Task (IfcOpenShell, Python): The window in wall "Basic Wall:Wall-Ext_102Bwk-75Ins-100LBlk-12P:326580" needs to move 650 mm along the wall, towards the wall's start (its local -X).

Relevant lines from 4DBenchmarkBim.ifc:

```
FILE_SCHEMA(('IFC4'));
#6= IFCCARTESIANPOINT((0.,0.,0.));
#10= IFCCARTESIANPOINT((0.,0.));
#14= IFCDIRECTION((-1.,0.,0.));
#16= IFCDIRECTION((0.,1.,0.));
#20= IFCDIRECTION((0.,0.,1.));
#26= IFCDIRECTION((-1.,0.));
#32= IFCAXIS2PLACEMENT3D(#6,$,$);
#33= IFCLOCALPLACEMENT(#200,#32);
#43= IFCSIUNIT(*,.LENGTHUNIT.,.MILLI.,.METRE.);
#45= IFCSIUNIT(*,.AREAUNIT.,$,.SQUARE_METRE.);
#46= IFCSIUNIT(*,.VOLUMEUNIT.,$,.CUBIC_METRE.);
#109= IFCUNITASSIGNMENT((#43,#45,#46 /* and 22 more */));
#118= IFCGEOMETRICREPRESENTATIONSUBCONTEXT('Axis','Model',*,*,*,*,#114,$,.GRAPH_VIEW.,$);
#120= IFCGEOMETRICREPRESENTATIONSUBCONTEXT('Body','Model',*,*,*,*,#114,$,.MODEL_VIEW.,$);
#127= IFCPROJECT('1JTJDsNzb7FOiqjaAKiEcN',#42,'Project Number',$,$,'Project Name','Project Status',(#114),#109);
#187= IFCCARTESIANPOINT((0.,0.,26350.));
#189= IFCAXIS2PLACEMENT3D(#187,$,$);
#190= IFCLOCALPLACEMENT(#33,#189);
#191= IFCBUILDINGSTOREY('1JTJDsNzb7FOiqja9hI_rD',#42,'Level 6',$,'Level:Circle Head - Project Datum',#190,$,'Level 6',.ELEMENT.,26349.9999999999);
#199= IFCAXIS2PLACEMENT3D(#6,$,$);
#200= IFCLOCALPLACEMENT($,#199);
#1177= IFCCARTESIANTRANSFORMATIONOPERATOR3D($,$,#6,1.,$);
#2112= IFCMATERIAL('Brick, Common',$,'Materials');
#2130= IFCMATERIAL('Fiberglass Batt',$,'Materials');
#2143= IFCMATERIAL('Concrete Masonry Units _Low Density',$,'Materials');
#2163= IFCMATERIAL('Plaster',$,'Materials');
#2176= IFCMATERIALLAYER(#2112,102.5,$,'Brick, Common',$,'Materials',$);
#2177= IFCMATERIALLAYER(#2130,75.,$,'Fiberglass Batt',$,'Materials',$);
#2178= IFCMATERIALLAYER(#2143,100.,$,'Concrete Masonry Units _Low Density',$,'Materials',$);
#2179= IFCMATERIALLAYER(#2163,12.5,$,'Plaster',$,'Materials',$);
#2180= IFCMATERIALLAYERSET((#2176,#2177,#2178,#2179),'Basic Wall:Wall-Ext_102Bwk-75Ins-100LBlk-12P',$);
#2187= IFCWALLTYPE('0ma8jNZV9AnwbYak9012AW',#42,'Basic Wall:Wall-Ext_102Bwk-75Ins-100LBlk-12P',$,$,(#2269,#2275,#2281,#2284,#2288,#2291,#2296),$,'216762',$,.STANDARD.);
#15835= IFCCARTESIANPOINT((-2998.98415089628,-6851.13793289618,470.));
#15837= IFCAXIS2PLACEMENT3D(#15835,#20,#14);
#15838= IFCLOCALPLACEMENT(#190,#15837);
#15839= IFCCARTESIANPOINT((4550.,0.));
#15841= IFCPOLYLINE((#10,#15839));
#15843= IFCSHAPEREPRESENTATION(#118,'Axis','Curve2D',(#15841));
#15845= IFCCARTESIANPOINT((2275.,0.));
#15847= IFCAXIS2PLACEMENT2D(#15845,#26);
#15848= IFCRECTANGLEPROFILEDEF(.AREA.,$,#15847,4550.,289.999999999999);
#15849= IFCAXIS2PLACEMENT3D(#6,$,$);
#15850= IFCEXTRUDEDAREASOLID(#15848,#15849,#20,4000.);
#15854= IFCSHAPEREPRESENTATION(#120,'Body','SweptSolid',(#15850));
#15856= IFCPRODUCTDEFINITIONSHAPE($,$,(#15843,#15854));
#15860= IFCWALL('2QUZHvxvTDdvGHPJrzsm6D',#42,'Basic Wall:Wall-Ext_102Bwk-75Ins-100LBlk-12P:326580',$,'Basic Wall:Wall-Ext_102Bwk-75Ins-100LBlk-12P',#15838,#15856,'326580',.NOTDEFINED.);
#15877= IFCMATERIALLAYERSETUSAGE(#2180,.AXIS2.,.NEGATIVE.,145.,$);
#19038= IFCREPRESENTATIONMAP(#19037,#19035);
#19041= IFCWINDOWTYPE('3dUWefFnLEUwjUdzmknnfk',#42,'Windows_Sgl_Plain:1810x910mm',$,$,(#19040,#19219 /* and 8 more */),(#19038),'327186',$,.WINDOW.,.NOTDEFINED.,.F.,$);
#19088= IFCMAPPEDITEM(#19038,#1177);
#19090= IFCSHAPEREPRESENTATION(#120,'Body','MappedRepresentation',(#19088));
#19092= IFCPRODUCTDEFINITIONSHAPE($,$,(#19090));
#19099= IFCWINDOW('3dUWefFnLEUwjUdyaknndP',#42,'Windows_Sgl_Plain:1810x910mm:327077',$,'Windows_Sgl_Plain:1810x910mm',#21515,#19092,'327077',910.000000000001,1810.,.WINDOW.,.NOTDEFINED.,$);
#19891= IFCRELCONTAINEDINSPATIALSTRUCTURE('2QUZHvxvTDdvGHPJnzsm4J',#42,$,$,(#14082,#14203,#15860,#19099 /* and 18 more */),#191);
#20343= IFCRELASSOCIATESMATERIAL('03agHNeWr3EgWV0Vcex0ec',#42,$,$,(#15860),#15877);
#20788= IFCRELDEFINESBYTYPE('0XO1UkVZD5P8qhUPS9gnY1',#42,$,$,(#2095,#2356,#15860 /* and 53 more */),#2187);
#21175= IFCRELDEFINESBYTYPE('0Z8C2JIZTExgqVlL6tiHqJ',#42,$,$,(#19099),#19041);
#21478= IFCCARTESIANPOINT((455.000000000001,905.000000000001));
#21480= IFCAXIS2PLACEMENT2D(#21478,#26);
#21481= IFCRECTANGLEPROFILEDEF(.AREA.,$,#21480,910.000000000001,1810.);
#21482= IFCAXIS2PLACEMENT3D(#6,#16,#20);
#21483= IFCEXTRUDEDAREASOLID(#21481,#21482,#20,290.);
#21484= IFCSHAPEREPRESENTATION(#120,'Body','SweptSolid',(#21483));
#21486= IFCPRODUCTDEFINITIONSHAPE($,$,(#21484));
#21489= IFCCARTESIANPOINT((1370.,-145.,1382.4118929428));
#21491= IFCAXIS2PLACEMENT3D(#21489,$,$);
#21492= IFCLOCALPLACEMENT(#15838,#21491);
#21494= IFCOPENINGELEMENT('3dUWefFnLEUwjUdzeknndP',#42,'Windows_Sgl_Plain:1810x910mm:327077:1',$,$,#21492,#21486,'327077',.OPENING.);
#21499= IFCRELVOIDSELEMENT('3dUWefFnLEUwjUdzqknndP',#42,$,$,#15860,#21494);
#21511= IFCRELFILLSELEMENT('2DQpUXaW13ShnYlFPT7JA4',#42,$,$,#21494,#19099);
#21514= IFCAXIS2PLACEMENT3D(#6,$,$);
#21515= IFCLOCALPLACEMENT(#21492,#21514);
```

```python
import ifcopenshell
import ifcopenshell.api.geometry
import ifcopenshell.util.placement

model = ifcopenshell.open("4DBenchmarkBim.ifc")

window = model.by_guid("3dUWefFnLEUwjUdyaknndP")
opening = window.FillsVoids[0].RelatingOpeningElement
wall = opening.VoidsElements[0].RelatingBuildingElement

wall_matrix = ifcopenshell.util.placement.get_local_placement(wall.ObjectPlacement)
shift = wall_matrix[:3, 0] * -650.0
before = ifcopenshell.util.placement.get_local_placement(window.ObjectPlacement)[:3, 3].copy()

# The window is placed relative to its opening, so it follows when the opening moves.
matrix = ifcopenshell.util.placement.get_local_placement(opening.ObjectPlacement)
matrix[:3, 3] += shift
ifcopenshell.api.geometry.edit_object_placement(
    model, product=opening, matrix=matrix, is_si=False, should_transform_children=True
)

after = ifcopenshell.util.placement.get_local_placement(window.ObjectPlacement)[:3, 3]
print("window moved by", (after - before).round(3) + 0.0)

model.write("4DBenchmarkBim_updated.ifc")
```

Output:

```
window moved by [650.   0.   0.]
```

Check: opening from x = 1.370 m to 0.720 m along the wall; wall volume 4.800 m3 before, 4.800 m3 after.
